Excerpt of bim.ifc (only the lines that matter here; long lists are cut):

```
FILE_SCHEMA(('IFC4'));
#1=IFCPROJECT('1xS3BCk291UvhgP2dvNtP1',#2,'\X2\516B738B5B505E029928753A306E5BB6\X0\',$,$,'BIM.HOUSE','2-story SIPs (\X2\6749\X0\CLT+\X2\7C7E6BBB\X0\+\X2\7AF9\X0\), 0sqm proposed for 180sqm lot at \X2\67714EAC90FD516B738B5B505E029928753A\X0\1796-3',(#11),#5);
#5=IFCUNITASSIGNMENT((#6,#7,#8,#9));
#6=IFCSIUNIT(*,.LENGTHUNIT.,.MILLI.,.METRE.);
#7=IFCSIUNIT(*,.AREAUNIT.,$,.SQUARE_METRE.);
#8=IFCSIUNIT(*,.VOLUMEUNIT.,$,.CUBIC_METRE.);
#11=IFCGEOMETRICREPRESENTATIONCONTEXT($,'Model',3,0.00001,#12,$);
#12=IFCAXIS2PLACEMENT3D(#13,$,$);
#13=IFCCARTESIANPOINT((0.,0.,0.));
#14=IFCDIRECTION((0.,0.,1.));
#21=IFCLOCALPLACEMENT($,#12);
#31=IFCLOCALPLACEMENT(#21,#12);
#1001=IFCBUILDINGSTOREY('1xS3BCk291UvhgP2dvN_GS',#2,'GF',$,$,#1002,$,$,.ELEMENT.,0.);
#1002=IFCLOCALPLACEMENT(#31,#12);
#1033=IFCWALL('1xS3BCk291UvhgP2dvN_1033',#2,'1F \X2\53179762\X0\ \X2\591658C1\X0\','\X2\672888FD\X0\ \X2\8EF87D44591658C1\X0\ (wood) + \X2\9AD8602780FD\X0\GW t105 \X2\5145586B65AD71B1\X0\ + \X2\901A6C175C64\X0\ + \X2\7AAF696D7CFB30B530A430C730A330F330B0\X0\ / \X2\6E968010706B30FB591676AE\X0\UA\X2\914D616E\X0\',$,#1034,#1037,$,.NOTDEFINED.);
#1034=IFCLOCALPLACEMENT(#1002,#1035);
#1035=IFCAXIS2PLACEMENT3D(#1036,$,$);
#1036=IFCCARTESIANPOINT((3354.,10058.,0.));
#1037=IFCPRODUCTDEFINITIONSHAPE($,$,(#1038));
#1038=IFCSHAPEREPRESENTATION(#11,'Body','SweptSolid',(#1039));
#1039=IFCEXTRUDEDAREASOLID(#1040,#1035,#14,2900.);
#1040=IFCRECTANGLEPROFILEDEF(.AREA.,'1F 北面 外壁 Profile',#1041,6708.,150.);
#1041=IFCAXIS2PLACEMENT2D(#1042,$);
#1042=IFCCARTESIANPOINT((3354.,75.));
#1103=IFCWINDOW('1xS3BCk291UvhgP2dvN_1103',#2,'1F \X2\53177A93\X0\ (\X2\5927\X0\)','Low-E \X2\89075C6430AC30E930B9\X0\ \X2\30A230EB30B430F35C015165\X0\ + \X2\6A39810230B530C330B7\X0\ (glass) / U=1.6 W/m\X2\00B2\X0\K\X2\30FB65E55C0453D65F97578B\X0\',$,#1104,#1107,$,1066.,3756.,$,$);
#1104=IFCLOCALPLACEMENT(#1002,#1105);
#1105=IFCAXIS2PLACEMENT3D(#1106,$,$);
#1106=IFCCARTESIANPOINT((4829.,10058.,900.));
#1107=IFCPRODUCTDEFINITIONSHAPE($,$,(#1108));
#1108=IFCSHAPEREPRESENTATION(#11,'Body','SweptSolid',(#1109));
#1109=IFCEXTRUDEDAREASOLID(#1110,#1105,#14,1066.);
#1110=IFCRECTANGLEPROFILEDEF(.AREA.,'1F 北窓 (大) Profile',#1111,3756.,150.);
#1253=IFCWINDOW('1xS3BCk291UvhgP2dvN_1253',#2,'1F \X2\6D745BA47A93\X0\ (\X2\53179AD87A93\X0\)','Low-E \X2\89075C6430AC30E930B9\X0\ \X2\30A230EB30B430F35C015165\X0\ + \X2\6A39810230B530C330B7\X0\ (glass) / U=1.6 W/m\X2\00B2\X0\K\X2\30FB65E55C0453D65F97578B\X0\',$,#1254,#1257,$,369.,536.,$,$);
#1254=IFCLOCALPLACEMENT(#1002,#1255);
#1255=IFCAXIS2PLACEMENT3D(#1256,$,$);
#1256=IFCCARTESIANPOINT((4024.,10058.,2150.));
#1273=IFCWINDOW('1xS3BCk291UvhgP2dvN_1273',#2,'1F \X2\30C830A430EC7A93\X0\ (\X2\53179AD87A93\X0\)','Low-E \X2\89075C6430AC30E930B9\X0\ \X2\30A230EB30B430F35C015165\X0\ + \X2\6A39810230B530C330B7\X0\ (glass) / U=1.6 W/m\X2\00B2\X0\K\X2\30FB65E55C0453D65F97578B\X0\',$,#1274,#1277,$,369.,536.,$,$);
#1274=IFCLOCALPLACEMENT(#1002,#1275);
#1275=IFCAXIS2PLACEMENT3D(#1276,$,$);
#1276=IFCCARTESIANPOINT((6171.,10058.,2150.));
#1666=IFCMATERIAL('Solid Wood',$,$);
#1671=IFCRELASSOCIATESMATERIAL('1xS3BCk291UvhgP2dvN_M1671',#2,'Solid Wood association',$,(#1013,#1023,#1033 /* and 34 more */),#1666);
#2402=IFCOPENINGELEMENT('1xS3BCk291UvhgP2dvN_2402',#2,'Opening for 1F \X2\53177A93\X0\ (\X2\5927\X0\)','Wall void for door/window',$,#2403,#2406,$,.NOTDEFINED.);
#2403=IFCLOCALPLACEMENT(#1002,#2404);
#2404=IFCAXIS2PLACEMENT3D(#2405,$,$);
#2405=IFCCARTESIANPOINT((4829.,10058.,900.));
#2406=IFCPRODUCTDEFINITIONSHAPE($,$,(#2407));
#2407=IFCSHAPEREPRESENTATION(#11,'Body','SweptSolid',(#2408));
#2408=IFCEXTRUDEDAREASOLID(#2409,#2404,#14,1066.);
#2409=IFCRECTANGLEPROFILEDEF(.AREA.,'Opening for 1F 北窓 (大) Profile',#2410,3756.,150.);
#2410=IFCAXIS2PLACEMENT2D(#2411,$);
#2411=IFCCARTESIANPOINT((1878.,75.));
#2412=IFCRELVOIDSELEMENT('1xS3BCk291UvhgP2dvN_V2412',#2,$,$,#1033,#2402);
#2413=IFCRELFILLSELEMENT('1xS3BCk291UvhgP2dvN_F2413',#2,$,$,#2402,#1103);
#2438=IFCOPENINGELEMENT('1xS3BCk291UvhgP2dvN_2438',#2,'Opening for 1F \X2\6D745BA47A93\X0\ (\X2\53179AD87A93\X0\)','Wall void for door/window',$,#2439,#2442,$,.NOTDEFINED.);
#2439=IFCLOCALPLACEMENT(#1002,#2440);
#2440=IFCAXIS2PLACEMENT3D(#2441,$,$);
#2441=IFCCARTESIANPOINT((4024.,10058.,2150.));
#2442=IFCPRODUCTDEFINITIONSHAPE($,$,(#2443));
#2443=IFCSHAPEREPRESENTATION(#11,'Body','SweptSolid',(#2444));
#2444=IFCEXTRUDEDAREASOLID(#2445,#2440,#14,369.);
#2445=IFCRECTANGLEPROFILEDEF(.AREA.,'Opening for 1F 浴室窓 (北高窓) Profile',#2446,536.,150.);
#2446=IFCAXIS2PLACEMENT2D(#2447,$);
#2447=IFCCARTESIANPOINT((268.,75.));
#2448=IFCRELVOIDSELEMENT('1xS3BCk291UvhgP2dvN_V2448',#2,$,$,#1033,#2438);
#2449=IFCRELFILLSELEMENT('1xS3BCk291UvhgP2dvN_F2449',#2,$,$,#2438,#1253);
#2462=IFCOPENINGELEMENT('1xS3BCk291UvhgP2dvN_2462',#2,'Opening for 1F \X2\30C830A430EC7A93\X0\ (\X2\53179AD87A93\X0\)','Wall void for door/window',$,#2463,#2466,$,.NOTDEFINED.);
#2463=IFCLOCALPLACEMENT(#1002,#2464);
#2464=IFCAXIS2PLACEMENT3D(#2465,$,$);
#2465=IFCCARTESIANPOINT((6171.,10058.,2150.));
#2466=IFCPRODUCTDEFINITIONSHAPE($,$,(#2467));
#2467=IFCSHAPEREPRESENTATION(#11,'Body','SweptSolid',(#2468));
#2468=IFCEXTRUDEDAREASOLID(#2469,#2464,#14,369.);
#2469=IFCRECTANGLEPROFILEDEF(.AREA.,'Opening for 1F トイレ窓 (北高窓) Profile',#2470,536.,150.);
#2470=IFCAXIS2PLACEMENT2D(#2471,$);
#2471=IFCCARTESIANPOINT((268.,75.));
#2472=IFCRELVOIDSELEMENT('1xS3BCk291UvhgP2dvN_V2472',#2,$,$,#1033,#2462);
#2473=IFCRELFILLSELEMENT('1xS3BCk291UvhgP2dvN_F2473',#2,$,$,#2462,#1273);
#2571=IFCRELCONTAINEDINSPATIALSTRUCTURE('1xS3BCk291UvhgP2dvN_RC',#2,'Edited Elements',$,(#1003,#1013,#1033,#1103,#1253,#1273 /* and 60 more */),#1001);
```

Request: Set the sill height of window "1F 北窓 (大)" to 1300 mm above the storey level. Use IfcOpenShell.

```python
import numpy as np
import ifcopenshell
import ifcopenshell.api.geometry
import ifcopenshell.geom
import ifcopenshell.util.element
import ifcopenshell.util.placement
import ifcopenshell.util.shape
import ifcopenshell.util.unit

model = ifcopenshell.open("bim.ifc")
unit_scale = ifcopenshell.util.unit.calculate_unit_scale(model)

window = model.by_id(1103)
opening = window.FillsVoids[0].RelatingOpeningElement
storey = ifcopenshell.util.element.get_container(window, ifc_class="IfcBuildingStorey")
level = ifcopenshell.util.placement.get_local_placement(storey.ObjectPlacement)[2, 3]

# The opening's origin need not be at the sill, so measure its lowest point.
shape = ifcopenshell.geom.create_shape(ifcopenshell.geom.settings(), opening)
bottom = ifcopenshell.util.shape.get_shape_bottom_elevation(shape, shape.geometry) / unit_scale
dz = level + 1.3 / unit_scale - bottom

shift = np.array([0.0, 0.0, dz])
# The window is not placed relative to its opening, so move both.
for product in (opening, window):
    matrix = ifcopenshell.util.placement.get_local_placement(product.ObjectPlacement)
    matrix[:3, 3] += shift
    ifcopenshell.api.geometry.edit_object_placement(model, product=product, matrix=matrix, is_si=False)

print(f"moved by {dz * unit_scale:+.3f} m")

model.write("bim_v2.ifc")
```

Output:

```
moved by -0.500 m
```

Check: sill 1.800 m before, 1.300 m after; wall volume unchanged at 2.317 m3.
